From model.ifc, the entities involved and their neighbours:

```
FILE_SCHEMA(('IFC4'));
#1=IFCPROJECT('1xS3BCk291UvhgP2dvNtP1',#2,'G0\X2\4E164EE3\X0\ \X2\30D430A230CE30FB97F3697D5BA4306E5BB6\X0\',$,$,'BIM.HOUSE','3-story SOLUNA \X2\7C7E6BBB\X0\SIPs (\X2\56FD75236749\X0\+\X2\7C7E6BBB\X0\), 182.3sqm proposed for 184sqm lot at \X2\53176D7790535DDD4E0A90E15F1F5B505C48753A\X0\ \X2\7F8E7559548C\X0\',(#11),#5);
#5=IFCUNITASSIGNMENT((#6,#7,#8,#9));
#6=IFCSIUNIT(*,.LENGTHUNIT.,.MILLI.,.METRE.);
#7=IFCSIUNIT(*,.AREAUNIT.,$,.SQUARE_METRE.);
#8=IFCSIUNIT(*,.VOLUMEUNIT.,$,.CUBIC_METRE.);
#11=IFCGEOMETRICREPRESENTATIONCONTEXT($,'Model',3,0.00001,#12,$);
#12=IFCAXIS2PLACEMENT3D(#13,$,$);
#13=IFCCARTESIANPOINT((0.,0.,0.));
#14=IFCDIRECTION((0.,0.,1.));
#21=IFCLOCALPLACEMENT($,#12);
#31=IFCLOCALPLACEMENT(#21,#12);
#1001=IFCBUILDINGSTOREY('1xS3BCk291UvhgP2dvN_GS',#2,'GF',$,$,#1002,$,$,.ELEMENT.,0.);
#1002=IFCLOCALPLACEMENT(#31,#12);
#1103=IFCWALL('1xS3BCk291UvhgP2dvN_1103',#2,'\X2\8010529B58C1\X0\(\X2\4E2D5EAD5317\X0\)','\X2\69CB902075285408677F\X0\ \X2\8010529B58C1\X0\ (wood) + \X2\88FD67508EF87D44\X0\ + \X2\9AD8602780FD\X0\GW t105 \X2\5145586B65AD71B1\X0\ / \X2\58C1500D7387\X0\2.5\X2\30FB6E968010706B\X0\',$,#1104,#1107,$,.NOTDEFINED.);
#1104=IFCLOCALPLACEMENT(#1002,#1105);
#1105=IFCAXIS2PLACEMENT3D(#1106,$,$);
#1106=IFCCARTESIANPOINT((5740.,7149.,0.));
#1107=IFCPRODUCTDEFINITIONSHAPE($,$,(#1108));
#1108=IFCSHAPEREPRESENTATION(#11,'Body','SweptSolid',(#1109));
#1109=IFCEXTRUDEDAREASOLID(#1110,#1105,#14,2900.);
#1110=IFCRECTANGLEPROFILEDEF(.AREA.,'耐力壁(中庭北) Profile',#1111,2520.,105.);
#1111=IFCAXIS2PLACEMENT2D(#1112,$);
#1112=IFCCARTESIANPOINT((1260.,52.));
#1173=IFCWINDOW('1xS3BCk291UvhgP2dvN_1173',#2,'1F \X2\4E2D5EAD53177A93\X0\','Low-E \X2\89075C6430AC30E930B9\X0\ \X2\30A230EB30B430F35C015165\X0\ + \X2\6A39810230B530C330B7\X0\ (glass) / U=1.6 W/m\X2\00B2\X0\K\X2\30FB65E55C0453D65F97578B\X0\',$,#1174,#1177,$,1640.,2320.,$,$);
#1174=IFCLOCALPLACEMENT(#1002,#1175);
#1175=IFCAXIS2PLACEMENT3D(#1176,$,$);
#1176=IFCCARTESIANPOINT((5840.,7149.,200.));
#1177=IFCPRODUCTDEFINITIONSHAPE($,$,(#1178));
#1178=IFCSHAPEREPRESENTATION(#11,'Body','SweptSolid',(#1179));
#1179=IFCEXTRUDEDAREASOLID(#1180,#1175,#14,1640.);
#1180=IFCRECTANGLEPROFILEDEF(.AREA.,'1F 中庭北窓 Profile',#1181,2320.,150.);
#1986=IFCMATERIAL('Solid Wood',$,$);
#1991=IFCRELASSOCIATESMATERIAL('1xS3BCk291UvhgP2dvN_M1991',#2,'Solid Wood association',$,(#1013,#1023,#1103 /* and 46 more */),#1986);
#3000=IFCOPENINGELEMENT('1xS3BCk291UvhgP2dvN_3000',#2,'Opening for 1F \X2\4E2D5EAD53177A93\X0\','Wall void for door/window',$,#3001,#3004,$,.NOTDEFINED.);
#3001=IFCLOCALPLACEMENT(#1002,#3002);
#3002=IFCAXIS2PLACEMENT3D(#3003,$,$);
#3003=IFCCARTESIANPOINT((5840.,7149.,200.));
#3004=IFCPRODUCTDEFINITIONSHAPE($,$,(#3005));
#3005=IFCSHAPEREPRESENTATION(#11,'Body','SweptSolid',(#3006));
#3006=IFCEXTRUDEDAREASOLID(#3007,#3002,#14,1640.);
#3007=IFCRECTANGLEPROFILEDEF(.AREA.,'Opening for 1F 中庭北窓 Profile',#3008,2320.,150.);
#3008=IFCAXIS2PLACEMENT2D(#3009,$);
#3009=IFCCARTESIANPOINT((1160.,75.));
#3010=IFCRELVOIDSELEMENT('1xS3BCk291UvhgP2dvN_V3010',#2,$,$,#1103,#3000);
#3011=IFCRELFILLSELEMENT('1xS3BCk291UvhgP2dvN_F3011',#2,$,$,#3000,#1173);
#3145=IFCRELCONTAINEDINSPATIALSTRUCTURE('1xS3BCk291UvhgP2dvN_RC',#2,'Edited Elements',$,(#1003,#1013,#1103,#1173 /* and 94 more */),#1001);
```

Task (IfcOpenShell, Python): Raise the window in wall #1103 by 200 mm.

```python
import numpy as np
import ifcopenshell
import ifcopenshell.api.geometry
import ifcopenshell.util.placement
import ifcopenshell.util.unit

model = ifcopenshell.open("model.ifc")
unit_scale = ifcopenshell.util.unit.calculate_unit_scale(model)

window = model.by_guid("1xS3BCk291UvhgP2dvN_1173")
opening = window.FillsVoids[0].RelatingOpeningElement
dz = 0.2 / unit_scale

shift = np.array([0.0, 0.0, dz])
# The window is not placed relative to its opening, so move both.
for product in (opening, window):
    matrix = ifcopenshell.util.placement.get_local_placement(product.ObjectPlacement)
    matrix[:3, 3] += shift
    ifcopenshell.api.geometry.edit_object_placement(model, product=product, matrix=matrix, is_si=False)

print(f"moved by {dz * unit_scale:+.3f} m")

model.write("model_edited.ifc")
```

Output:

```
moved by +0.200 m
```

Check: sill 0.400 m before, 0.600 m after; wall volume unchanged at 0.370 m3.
